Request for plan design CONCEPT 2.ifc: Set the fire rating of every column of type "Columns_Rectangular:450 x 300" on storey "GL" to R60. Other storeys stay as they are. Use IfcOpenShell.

First a look at what the model holds.

```python
import ifcopenshell
import ifcopenshell.util.element

model = ifcopenshell.open("plan design CONCEPT 2.ifc")
print(model.schema)
storey = next(s for s in model.by_type("IfcBuildingStorey") if s.Name == "GL")
columns = [e for e in ifcopenshell.util.element.get_decomposition(storey) if e.is_a("IfcColumn")]
seen = {}
for e in columns:
    element_type = ifcopenshell.util.element.get_type(e)
    key = (element_type.Name if element_type != e and element_type else None, ifcopenshell.util.element.get_pset(e, "Pset_ColumnCommon", "FireRating"))
    seen[key] = seen.get(key, 0) + 1
for (name, value), count in sorted(seen.items(), key=str):
    print(count, "x", name, "|", value)
```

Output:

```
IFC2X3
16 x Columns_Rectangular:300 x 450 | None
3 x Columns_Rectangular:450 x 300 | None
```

```python
import ifcopenshell
import ifcopenshell.api.pset
import ifcopenshell.util.element

model = ifcopenshell.open("plan design CONCEPT 2.ifc")

storey = next(s for s in model.by_type("IfcBuildingStorey") if s.Name == "GL")
columns = [e for e in ifcopenshell.util.element.get_decomposition(storey) if e.is_a("IfcColumn")]

count = 0
for e in columns:
    element_type = ifcopenshell.util.element.get_type(e)
    if element_type in (None, e) or element_type.Name != "Columns_Rectangular:450 x 300":
        continue
    # add_pset returns the element's existing set when there is one.
    pset = ifcopenshell.api.pset.add_pset(model, product=e, name="Pset_ColumnCommon")
    ifcopenshell.api.pset.edit_pset(model, pset=pset, properties={"FireRating": "R60"})
    count += 1

print(count, "columns updated")

model.write("plan design CONCEPT 2-out.ifc")
```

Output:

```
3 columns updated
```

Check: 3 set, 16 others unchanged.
